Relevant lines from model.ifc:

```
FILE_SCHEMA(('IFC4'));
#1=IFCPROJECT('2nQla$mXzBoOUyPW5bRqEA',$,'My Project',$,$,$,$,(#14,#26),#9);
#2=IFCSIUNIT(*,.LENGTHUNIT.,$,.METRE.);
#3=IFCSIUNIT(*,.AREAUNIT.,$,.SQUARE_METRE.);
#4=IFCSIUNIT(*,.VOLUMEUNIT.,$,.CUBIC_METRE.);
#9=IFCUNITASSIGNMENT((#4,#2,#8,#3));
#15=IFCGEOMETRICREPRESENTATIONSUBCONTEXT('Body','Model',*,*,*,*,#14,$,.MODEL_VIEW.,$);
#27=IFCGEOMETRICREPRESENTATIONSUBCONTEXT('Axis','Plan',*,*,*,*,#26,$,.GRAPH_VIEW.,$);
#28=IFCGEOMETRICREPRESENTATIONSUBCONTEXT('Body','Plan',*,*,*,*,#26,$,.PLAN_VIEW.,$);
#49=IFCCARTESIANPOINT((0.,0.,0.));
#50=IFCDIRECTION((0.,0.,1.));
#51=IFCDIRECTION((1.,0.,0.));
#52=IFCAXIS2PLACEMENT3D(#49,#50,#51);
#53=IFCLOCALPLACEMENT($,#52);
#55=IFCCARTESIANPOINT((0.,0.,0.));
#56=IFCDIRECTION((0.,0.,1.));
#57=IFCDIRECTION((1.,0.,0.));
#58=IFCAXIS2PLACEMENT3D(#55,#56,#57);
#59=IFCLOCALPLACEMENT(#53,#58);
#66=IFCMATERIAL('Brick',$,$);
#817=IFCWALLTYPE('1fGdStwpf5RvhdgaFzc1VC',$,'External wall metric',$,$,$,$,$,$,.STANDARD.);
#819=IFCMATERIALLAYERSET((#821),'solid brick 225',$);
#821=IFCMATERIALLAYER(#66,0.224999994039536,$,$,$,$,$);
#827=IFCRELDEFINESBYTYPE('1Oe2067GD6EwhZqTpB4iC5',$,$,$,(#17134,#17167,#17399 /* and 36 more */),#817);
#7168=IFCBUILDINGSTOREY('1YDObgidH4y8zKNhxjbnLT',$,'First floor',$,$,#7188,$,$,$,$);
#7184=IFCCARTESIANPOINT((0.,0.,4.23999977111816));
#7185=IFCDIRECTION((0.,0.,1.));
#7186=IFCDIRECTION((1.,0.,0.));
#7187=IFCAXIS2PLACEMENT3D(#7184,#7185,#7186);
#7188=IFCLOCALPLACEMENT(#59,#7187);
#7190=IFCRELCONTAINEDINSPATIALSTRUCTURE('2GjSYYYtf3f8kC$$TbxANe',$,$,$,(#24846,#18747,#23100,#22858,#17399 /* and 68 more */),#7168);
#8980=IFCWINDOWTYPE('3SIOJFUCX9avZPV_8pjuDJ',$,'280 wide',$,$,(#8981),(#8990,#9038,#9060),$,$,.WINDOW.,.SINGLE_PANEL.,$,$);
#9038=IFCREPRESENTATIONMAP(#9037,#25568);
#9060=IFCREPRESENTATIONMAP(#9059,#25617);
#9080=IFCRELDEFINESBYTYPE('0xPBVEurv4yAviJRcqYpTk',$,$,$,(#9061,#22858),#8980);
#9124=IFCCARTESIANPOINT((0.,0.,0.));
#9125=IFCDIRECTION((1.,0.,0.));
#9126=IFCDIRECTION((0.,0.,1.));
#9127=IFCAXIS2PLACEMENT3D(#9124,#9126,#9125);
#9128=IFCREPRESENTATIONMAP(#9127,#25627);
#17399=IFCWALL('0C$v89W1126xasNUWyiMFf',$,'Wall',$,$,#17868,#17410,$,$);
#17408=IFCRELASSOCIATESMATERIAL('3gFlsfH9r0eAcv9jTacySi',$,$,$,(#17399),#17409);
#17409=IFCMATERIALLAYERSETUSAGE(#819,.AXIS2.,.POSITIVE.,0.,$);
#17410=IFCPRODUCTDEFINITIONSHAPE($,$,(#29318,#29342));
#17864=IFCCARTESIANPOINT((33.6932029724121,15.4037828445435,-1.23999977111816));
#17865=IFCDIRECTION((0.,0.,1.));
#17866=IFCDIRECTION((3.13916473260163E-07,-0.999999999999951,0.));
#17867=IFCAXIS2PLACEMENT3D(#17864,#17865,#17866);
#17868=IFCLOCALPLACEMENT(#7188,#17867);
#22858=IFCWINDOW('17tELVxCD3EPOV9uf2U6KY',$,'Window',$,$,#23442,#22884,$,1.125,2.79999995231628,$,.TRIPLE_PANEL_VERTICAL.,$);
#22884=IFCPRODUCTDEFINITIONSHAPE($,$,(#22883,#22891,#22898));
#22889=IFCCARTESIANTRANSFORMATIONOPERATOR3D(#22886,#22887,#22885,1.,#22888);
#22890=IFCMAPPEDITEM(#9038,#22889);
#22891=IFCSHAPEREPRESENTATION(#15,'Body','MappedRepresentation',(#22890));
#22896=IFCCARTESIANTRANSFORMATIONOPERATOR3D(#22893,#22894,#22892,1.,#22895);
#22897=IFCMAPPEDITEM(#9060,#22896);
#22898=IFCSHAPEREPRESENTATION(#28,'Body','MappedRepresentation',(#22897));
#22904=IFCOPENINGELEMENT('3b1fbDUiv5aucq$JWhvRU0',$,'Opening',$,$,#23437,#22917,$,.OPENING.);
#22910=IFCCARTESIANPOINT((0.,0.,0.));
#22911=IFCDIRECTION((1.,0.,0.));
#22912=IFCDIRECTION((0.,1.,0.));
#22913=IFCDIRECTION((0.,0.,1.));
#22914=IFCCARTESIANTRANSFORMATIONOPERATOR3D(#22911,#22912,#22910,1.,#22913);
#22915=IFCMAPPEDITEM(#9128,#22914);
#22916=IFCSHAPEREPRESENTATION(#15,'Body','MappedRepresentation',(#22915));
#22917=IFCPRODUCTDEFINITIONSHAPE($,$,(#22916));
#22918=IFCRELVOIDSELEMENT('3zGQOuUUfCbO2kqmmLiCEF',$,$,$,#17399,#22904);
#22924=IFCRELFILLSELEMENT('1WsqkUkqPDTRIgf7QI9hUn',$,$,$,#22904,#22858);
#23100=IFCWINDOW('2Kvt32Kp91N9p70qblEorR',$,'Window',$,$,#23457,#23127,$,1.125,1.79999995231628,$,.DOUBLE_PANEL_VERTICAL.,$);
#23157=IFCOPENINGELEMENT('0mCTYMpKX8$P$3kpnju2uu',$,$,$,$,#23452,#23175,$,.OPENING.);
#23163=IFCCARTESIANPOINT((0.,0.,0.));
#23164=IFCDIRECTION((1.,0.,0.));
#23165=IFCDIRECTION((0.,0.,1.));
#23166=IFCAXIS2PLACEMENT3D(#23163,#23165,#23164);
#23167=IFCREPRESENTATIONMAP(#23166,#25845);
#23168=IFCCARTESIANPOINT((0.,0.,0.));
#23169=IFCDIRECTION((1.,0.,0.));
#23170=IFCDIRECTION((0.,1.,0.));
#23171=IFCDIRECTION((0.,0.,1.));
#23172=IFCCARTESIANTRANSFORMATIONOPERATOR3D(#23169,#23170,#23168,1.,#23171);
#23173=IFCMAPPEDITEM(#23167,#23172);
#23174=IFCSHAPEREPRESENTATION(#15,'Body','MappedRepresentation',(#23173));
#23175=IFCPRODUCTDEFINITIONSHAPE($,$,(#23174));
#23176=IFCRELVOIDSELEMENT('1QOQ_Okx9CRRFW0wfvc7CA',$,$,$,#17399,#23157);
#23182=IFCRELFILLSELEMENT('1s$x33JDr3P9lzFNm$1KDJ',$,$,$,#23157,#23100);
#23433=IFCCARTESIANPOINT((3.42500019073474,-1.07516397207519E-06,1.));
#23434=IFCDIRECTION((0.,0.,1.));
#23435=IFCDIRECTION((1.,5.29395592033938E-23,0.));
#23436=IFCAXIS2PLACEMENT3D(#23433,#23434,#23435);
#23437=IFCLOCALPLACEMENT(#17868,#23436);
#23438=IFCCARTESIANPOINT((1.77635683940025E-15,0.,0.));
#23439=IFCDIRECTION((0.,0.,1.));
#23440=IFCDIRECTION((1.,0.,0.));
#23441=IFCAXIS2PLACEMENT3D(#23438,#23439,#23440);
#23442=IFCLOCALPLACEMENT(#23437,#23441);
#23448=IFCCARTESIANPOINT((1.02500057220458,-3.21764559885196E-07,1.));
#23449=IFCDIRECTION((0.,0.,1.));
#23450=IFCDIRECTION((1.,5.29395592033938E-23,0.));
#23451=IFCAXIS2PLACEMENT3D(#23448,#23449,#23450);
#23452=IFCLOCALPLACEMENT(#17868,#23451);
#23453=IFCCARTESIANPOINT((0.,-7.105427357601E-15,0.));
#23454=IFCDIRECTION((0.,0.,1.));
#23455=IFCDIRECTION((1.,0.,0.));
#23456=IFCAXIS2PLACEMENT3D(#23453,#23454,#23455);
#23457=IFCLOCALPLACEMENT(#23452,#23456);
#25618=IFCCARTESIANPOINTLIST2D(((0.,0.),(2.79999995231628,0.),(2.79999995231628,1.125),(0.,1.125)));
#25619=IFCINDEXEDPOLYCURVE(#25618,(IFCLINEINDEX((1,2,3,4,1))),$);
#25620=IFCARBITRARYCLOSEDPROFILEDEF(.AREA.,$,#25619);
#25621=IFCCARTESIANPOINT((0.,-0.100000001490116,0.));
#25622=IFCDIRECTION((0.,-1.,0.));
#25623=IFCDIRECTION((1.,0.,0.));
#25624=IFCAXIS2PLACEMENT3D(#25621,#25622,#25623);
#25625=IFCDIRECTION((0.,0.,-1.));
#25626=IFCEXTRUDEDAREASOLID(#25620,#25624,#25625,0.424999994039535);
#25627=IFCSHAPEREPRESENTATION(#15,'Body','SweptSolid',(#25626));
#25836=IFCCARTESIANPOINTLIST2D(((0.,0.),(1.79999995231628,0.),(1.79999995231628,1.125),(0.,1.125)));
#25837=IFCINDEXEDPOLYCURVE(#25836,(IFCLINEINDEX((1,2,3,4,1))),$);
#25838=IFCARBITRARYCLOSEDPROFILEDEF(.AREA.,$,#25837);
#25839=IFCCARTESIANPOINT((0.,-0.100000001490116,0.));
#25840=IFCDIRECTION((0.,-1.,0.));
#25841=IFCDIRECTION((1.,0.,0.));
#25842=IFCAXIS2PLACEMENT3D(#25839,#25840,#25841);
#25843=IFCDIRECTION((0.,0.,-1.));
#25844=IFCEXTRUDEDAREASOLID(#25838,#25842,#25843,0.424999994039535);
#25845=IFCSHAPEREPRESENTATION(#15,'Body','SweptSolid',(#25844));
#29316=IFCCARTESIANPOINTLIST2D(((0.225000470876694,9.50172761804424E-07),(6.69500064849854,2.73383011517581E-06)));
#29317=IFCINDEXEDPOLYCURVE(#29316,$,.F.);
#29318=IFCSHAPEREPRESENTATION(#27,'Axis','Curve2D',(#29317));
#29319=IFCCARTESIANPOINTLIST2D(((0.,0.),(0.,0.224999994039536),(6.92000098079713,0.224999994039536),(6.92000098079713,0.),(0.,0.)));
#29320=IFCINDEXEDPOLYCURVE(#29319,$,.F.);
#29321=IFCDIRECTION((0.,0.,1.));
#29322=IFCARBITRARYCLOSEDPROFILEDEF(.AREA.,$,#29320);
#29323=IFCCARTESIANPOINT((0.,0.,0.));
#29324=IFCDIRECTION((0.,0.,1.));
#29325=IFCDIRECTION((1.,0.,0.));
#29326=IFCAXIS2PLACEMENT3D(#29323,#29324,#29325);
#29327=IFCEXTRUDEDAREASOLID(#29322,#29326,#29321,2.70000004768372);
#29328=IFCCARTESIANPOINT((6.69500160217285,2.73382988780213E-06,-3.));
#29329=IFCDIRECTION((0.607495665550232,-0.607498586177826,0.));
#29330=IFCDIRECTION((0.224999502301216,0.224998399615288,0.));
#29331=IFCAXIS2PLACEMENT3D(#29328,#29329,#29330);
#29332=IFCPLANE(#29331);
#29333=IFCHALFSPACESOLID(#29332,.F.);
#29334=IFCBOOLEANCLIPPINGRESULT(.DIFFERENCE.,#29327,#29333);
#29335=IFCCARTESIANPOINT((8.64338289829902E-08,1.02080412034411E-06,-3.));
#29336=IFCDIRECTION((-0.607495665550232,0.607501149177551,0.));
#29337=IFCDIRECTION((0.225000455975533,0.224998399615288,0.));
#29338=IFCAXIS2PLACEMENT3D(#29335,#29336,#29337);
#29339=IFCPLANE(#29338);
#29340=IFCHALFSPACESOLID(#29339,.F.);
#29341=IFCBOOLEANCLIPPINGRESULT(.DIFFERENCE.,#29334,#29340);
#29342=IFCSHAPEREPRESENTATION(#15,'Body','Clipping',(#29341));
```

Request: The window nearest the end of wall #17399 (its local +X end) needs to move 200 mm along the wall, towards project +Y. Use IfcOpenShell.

```python
import ifcopenshell
import ifcopenshell.api.geometry
import ifcopenshell.util.placement

model = ifcopenshell.open("model.ifc")

window = model.by_id(22858)
opening = window.FillsVoids[0].RelatingOpeningElement
wall = opening.VoidsElements[0].RelatingBuildingElement

wall_matrix = ifcopenshell.util.placement.get_local_placement(wall.ObjectPlacement)
shift = wall_matrix[:3, 0] * -0.2
before = ifcopenshell.util.placement.get_local_placement(window.ObjectPlacement)[:3, 3].copy()

# The window is placed relative to its opening, so it follows when the opening moves.
matrix = ifcopenshell.util.placement.get_local_placement(opening.ObjectPlacement)
matrix[:3, 3] += shift
ifcopenshell.api.geometry.edit_object_placement(
    model, product=opening, matrix=matrix, is_si=False, should_transform_children=True
)

after = ifcopenshell.util.placement.get_local_placement(window.ObjectPlacement)[:3, 3]
print("window moved by", (after - before).round(3) + 0.0)

model.write("model_v2.ifc")
```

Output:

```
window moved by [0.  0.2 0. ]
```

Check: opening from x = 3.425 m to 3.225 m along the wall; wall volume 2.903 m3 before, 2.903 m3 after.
